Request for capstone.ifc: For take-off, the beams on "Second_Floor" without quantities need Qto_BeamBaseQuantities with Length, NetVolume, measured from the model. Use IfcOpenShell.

First a look at what the model holds.

```python
import ifcopenshell
import ifcopenshell.util.element
import ifcopenshell.util.unit

model = ifcopenshell.open("capstone.ifc")
print(model.schema)
for unit_type in ("LENGTHUNIT", "AREAUNIT", "VOLUMEUNIT"):
    print(unit_type, ifcopenshell.util.unit.calculate_unit_scale(model, unit_type))
storey = next(s for s in model.by_type("IfcBuildingStorey") if s.Name == "Second_Floor")
beams = [e for e in ifcopenshell.util.element.get_decomposition(storey) if e.is_a("IfcBeam")]
for e in sorted(beams, key=lambda e: e.id()):
    print(e.id(), e.is_a(), e.Name, list(ifcopenshell.util.element.get_psets(e, qtos_only=True)), sep=" | ")
```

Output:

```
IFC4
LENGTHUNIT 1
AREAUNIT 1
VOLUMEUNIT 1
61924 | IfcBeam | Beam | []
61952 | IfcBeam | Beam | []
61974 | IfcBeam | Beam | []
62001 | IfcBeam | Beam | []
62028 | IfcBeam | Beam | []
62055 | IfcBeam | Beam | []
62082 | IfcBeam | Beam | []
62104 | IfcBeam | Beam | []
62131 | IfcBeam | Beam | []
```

```python
import ifcopenshell
import ifcopenshell.api.pset
import ifcopenshell.geom
import ifcopenshell.util.element
import ifcopenshell.util.shape
import ifcopenshell.util.unit

model = ifcopenshell.open("capstone.ifc")
unit_scale = ifcopenshell.util.unit.calculate_unit_scale(model)
volume_scale = ifcopenshell.util.unit.calculate_unit_scale(model, "VOLUMEUNIT")
settings = ifcopenshell.geom.settings()

storey = next(s for s in model.by_type("IfcBuildingStorey") if s.Name == "Second_Floor")
beams = [e for e in ifcopenshell.util.element.get_decomposition(storey) if e.is_a("IfcBeam")]

for e in sorted(beams, key=lambda e: e.id()):
    if ifcopenshell.util.element.get_psets(e, qtos_only=True, should_inherit=False):
        continue
    # Geometry comes back in metres, in the element's own axes.
    shape = ifcopenshell.geom.create_shape(settings, e)
    values = {
        "Length": ifcopenshell.util.shape.get_max_xyz(shape.geometry) / unit_scale,
        "NetVolume": ifcopenshell.util.shape.get_volume(shape.geometry) / volume_scale,
    }
    qto = ifcopenshell.api.pset.add_qto(model, product=e, name="Qto_BeamBaseQuantities")
    ifcopenshell.api.pset.edit_qto(model, qto=qto, properties=values)
    print(e.id(), {k: round(v, 3) for k, v in values.items()})

model.write("capstone_edited.ifc")
```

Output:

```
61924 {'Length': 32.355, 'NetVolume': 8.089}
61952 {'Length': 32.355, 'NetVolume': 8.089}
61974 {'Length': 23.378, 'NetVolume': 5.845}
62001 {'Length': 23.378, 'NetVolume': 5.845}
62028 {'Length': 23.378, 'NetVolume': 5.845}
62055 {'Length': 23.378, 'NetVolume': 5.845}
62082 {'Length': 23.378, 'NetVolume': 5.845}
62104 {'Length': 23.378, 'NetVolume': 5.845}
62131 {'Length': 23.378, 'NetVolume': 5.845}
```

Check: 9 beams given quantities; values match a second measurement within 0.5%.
